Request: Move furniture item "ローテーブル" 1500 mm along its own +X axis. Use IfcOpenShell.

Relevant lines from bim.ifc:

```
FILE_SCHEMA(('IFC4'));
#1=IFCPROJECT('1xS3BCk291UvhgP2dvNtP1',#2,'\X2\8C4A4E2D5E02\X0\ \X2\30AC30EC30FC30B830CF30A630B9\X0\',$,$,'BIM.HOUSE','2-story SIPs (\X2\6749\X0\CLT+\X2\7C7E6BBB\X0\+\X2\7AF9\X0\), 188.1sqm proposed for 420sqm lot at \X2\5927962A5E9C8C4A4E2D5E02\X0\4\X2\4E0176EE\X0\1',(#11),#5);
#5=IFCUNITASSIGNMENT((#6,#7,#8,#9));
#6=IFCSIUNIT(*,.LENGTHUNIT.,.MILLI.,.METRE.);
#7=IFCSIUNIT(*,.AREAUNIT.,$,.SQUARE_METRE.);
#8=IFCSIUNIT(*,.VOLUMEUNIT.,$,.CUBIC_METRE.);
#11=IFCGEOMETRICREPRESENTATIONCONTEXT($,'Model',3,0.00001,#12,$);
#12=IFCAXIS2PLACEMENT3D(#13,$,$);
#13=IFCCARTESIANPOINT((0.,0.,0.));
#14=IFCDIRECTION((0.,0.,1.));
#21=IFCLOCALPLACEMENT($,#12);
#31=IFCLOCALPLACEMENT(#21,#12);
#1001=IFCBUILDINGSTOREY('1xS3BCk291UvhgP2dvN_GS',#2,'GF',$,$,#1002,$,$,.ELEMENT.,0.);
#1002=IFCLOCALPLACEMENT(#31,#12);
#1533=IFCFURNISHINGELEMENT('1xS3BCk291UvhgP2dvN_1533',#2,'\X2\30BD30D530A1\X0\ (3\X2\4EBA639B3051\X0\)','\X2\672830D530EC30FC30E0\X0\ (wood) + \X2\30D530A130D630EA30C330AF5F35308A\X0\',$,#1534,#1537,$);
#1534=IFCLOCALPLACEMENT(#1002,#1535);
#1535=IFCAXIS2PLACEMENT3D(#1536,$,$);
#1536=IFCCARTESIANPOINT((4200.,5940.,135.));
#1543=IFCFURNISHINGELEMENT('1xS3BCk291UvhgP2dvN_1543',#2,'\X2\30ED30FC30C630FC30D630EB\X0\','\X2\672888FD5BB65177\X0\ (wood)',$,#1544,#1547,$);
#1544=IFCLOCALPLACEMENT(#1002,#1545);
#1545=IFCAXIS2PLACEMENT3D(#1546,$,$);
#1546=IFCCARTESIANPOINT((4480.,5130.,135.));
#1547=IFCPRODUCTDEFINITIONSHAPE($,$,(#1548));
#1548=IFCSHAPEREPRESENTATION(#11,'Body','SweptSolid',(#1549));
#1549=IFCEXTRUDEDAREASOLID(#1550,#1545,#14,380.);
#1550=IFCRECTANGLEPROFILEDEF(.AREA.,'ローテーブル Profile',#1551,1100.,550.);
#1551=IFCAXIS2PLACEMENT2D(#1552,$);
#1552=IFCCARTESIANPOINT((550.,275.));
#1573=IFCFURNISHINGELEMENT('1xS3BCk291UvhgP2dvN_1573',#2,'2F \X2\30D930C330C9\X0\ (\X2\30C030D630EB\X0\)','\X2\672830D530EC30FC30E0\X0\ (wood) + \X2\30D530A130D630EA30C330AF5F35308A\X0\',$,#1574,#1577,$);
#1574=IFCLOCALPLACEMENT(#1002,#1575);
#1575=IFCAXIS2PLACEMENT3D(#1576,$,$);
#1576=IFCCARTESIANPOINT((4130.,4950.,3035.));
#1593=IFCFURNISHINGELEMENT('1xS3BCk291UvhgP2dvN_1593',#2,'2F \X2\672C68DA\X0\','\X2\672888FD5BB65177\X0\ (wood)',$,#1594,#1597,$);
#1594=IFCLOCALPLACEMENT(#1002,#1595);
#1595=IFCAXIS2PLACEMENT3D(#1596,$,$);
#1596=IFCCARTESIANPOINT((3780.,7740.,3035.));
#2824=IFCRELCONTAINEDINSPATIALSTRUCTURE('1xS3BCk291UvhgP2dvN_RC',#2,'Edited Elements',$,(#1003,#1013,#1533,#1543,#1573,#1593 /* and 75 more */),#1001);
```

```python
import ifcopenshell
import ifcopenshell.api.geometry
import ifcopenshell.util.placement
import ifcopenshell.util.unit

model = ifcopenshell.open("bim.ifc")
unit_scale = ifcopenshell.util.unit.calculate_unit_scale(model)

item = model.by_id(1543)
matrix = ifcopenshell.util.placement.get_local_placement(item.ObjectPlacement)
matrix[:3, 3] += matrix[:3, 0] * 1.5 / unit_scale
ifcopenshell.api.geometry.edit_object_placement(model, product=item, matrix=matrix, is_si=False)

print(ifcopenshell.util.placement.get_local_placement(item.ObjectPlacement).round(3) + 0.0)

model.write("bim_rev.ifc")
```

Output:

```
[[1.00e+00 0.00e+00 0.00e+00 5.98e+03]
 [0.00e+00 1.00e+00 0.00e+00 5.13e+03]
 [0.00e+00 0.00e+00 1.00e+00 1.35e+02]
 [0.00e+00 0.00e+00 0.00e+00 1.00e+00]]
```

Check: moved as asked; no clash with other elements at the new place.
